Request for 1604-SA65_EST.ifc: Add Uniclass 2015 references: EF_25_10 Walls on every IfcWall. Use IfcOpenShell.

First a look at what the model holds.

```python
import ifcopenshell

model = ifcopenshell.open("1604-SA65_EST.ifc")
print(model.schema)
print("classifications:", [c.Name for c in model.by_type("IfcClassification")])
for ifc_class in ("IfcDoor", "IfcRoof", "IfcStair", "IfcWall", "IfcWindow"):
    print(ifc_class, len(model.by_type(ifc_class)))
```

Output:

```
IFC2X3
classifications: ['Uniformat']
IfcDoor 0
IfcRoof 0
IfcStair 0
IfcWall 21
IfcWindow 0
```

```python
import ifcopenshell
import ifcopenshell.api.classification

model = ifcopenshell.open("1604-SA65_EST.ifc")

# IFC2X3 requires Source and Edition and has no link from the project to the system.
system = model.create_entity("IfcClassification", Source="NBS", Edition="2015", Name="Uniclass 2015")

codes = {
    "IfcWall": ("EF_25_10", "Walls"),
}
for ifc_class, (code, name) in codes.items():
    products = model.by_type(ifc_class)
    ifcopenshell.api.classification.add_reference(
        model, products=products, classification=system, identification=code, name=name
    )
    print(code, len(products))

model.write("1604-SA65_EST_edited.ifc")
```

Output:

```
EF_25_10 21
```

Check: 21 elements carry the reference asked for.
